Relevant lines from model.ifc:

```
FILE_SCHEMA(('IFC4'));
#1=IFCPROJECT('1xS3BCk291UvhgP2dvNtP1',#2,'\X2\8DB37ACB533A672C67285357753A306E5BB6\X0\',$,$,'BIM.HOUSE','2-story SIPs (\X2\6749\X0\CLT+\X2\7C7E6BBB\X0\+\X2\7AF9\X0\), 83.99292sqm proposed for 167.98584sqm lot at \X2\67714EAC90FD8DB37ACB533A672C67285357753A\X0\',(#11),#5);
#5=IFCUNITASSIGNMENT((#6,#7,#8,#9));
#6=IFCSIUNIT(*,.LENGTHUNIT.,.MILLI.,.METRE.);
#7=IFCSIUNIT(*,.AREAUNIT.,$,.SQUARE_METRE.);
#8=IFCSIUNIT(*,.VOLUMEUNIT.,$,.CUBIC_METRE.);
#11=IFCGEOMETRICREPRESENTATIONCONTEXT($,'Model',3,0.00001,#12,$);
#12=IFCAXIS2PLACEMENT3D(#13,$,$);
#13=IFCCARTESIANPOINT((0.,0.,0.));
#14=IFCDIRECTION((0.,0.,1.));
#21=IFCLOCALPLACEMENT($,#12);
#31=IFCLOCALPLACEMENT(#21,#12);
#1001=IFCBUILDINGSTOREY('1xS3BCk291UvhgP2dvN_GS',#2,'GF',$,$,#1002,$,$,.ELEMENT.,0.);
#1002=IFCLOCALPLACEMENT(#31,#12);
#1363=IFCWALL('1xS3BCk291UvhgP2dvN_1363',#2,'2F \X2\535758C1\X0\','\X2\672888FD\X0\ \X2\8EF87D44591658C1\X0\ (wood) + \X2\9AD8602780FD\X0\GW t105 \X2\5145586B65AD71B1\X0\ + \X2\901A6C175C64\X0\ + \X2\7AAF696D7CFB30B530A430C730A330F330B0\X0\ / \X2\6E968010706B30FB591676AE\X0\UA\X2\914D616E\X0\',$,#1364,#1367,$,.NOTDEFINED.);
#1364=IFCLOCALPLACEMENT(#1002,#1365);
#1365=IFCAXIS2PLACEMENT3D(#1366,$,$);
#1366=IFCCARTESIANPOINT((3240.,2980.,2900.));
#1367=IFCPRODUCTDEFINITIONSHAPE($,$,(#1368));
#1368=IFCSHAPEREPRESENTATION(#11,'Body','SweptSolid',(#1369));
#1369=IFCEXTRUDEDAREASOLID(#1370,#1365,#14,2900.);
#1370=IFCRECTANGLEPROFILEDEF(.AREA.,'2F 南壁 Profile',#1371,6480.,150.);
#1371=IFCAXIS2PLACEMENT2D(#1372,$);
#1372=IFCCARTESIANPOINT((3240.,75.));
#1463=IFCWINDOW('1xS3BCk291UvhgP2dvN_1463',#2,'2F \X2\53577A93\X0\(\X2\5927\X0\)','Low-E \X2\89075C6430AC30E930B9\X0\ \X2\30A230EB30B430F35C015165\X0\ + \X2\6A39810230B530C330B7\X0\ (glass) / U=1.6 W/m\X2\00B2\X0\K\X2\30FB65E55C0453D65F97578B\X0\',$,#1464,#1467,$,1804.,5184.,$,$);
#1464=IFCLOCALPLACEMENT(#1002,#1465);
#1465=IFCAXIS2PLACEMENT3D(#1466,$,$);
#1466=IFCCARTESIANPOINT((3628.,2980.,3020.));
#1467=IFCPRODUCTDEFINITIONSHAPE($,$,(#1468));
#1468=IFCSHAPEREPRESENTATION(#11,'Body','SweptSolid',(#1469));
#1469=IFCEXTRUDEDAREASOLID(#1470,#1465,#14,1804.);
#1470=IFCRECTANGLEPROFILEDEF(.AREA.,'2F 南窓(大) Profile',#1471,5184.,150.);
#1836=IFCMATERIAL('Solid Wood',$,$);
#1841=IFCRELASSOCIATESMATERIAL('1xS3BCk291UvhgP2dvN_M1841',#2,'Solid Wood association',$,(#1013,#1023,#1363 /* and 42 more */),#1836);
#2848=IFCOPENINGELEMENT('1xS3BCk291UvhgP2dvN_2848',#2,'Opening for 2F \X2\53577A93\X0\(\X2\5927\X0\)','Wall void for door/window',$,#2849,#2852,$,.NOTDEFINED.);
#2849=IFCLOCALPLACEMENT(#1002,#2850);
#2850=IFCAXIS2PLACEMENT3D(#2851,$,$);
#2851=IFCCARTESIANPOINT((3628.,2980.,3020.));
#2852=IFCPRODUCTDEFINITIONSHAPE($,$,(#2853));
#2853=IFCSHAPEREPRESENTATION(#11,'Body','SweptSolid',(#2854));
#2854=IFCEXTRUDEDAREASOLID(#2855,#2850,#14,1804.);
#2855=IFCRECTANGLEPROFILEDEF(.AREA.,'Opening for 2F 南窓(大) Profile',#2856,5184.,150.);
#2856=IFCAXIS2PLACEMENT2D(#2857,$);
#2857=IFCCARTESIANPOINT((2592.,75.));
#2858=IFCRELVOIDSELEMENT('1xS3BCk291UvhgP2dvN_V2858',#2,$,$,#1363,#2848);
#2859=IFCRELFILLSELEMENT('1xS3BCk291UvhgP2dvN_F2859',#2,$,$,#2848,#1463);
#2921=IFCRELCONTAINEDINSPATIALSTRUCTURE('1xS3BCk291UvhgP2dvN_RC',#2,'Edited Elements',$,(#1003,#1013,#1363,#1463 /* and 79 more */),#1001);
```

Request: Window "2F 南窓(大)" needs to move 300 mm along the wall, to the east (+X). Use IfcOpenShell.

```python
import ifcopenshell
import ifcopenshell.api.geometry
import ifcopenshell.util.placement
import ifcopenshell.util.unit

model = ifcopenshell.open("model.ifc")
unit_scale = ifcopenshell.util.unit.calculate_unit_scale(model)

window = model.by_guid("1xS3BCk291UvhgP2dvN_1463")
opening = window.FillsVoids[0].RelatingOpeningElement
wall = opening.VoidsElements[0].RelatingBuildingElement

wall_matrix = ifcopenshell.util.placement.get_local_placement(wall.ObjectPlacement)
shift = wall_matrix[:3, 0] * 0.3 / unit_scale
before = ifcopenshell.util.placement.get_local_placement(window.ObjectPlacement)[:3, 3].copy()

# The window is not placed relative to its opening, so move both.
for product in (opening, window):
    matrix = ifcopenshell.util.placement.get_local_placement(product.ObjectPlacement)
    matrix[:3, 3] += shift
    ifcopenshell.api.geometry.edit_object_placement(model, product=product, matrix=matrix, is_si=False)

after = ifcopenshell.util.placement.get_local_placement(window.ObjectPlacement)[:3, 3]
print("window moved by", (after - before).round(3) + 0.0)

model.write("model_rev.ifc")
```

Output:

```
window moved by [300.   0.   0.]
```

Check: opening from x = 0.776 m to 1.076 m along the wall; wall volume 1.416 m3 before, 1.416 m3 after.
